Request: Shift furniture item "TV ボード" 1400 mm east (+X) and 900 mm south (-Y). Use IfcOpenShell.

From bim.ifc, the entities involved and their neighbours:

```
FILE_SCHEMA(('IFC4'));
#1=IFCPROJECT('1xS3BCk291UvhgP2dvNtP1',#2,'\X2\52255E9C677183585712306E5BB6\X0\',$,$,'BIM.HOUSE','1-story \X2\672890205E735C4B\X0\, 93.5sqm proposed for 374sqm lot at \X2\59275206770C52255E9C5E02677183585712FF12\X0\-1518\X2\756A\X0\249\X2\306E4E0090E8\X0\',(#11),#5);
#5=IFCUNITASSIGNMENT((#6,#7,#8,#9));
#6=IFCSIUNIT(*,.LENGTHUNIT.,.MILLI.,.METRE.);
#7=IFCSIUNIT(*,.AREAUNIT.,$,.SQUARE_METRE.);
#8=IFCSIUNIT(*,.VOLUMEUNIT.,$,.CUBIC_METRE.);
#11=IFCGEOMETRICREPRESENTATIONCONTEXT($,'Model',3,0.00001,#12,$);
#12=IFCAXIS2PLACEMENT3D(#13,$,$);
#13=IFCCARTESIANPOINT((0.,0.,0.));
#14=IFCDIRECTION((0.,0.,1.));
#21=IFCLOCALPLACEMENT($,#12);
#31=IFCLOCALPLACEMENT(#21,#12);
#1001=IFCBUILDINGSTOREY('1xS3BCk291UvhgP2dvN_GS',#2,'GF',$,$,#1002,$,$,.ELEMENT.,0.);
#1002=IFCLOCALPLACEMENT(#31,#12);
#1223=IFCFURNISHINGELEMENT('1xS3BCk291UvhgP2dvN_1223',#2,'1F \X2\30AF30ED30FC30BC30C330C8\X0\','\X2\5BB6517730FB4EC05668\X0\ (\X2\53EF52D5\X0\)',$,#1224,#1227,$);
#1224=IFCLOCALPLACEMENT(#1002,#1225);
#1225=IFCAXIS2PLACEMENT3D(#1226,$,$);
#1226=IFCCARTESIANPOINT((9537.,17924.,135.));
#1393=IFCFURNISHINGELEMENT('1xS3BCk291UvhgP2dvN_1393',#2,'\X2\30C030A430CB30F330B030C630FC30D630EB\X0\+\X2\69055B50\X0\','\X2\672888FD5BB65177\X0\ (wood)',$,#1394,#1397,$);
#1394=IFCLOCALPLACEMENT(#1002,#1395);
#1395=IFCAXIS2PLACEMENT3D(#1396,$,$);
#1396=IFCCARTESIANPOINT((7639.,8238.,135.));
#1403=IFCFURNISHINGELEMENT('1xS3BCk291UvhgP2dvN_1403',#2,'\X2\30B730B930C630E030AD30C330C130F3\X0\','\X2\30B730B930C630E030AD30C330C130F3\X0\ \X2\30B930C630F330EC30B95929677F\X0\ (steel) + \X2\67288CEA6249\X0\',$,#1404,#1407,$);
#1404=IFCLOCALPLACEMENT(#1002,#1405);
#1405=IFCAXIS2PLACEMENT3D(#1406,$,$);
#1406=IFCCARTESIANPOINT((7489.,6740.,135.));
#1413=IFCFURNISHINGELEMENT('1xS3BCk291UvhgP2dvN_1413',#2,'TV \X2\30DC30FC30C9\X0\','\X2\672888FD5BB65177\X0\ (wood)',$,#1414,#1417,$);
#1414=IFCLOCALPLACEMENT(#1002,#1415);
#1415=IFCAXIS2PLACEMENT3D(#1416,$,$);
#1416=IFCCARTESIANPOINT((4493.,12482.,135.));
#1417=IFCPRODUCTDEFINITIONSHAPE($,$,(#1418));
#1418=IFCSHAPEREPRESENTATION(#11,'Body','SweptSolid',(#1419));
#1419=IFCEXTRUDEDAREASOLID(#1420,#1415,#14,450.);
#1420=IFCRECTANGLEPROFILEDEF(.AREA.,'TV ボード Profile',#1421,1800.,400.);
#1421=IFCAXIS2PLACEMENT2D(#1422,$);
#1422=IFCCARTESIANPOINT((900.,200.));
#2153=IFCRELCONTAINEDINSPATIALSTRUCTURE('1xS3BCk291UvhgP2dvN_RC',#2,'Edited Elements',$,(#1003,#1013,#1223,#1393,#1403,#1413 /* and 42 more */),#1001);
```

```python
import ifcopenshell
import ifcopenshell.api.geometry
import ifcopenshell.util.placement
import ifcopenshell.util.unit

model = ifcopenshell.open("bim.ifc")
unit_scale = ifcopenshell.util.unit.calculate_unit_scale(model)

item = model.by_guid("1xS3BCk291UvhgP2dvN_1413")
matrix = ifcopenshell.util.placement.get_local_placement(item.ObjectPlacement)
matrix[0, 3] += 1.4 / unit_scale
matrix[1, 3] -= 0.9 / unit_scale
ifcopenshell.api.geometry.edit_object_placement(model, product=item, matrix=matrix, is_si=False)

print(ifcopenshell.util.placement.get_local_placement(item.ObjectPlacement).round(3) + 0.0)

model.write("bim-out.ifc")
```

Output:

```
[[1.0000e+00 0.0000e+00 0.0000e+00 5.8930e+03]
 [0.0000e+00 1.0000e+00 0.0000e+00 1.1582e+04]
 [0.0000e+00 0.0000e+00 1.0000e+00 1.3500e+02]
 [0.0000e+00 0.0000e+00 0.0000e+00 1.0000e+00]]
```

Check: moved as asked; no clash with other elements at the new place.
